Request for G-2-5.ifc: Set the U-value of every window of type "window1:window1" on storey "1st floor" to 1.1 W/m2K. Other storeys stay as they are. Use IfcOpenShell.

First a look at what the model holds.

```python
import ifcopenshell
import ifcopenshell.util.element

model = ifcopenshell.open("G-2-5.ifc")
print(model.schema)
storey = next(s for s in model.by_type("IfcBuildingStorey") if s.Name == "1st floor")
windows = [e for e in ifcopenshell.util.element.get_decomposition(storey) if e.is_a("IfcWindow")]
seen = {}
for e in windows:
    element_type = ifcopenshell.util.element.get_type(e)
    key = (element_type.Name if element_type != e and element_type else None, ifcopenshell.util.element.get_pset(e, "Pset_WindowCommon", "ThermalTransmittance"))
    seen[key] = seen.get(key, 0) + 1
for (name, value), count in sorted(seen.items(), key=str):
    print(count, "x", name, "|", value)
```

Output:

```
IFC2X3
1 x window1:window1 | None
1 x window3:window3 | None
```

```python
import ifcopenshell
import ifcopenshell.api.pset
import ifcopenshell.util.element

model = ifcopenshell.open("G-2-5.ifc")

storey = next(s for s in model.by_type("IfcBuildingStorey") if s.Name == "1st floor")
windows = [e for e in ifcopenshell.util.element.get_decomposition(storey) if e.is_a("IfcWindow")]

count = 0
for e in windows:
    element_type = ifcopenshell.util.element.get_type(e)
    if element_type in (None, e) or element_type.Name != "window1:window1":
        continue
    # add_pset returns the element's existing set when there is one.
    pset = ifcopenshell.api.pset.add_pset(model, product=e, name="Pset_WindowCommon")
    ifcopenshell.api.pset.edit_pset(model, pset=pset, properties={"ThermalTransmittance": 1.1})
    count += 1

print(count, "windows updated")

model.write("G-2-5_rev.ifc")
```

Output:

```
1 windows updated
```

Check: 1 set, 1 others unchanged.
